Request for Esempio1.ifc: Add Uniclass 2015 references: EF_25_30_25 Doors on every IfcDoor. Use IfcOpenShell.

First a look at what the model holds.

```python
import ifcopenshell

model = ifcopenshell.open("Esempio1.ifc")
print(model.schema)
print("classifications:", [c.Name for c in model.by_type("IfcClassification")])
for ifc_class in ("IfcDoor", "IfcRoof", "IfcStair", "IfcWall", "IfcWindow"):
    print(ifc_class, len(model.by_type(ifc_class)))
```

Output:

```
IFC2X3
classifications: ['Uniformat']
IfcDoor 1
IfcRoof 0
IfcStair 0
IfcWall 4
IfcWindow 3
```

```python
import ifcopenshell
import ifcopenshell.api.classification

model = ifcopenshell.open("Esempio1.ifc")

# IFC2X3 requires Source and Edition and has no link from the project to the system.
system = model.create_entity("IfcClassification", Source="NBS", Edition="2015", Name="Uniclass 2015")

codes = {
    "IfcDoor": ("EF_25_30_25", "Doors"),
}
for ifc_class, (code, name) in codes.items():
    products = model.by_type(ifc_class)
    ifcopenshell.api.classification.add_reference(
        model, products=products, classification=system, identification=code, name=name
    )
    print(code, len(products))

model.write("Esempio1-out.ifc")
```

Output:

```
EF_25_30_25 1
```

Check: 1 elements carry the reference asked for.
